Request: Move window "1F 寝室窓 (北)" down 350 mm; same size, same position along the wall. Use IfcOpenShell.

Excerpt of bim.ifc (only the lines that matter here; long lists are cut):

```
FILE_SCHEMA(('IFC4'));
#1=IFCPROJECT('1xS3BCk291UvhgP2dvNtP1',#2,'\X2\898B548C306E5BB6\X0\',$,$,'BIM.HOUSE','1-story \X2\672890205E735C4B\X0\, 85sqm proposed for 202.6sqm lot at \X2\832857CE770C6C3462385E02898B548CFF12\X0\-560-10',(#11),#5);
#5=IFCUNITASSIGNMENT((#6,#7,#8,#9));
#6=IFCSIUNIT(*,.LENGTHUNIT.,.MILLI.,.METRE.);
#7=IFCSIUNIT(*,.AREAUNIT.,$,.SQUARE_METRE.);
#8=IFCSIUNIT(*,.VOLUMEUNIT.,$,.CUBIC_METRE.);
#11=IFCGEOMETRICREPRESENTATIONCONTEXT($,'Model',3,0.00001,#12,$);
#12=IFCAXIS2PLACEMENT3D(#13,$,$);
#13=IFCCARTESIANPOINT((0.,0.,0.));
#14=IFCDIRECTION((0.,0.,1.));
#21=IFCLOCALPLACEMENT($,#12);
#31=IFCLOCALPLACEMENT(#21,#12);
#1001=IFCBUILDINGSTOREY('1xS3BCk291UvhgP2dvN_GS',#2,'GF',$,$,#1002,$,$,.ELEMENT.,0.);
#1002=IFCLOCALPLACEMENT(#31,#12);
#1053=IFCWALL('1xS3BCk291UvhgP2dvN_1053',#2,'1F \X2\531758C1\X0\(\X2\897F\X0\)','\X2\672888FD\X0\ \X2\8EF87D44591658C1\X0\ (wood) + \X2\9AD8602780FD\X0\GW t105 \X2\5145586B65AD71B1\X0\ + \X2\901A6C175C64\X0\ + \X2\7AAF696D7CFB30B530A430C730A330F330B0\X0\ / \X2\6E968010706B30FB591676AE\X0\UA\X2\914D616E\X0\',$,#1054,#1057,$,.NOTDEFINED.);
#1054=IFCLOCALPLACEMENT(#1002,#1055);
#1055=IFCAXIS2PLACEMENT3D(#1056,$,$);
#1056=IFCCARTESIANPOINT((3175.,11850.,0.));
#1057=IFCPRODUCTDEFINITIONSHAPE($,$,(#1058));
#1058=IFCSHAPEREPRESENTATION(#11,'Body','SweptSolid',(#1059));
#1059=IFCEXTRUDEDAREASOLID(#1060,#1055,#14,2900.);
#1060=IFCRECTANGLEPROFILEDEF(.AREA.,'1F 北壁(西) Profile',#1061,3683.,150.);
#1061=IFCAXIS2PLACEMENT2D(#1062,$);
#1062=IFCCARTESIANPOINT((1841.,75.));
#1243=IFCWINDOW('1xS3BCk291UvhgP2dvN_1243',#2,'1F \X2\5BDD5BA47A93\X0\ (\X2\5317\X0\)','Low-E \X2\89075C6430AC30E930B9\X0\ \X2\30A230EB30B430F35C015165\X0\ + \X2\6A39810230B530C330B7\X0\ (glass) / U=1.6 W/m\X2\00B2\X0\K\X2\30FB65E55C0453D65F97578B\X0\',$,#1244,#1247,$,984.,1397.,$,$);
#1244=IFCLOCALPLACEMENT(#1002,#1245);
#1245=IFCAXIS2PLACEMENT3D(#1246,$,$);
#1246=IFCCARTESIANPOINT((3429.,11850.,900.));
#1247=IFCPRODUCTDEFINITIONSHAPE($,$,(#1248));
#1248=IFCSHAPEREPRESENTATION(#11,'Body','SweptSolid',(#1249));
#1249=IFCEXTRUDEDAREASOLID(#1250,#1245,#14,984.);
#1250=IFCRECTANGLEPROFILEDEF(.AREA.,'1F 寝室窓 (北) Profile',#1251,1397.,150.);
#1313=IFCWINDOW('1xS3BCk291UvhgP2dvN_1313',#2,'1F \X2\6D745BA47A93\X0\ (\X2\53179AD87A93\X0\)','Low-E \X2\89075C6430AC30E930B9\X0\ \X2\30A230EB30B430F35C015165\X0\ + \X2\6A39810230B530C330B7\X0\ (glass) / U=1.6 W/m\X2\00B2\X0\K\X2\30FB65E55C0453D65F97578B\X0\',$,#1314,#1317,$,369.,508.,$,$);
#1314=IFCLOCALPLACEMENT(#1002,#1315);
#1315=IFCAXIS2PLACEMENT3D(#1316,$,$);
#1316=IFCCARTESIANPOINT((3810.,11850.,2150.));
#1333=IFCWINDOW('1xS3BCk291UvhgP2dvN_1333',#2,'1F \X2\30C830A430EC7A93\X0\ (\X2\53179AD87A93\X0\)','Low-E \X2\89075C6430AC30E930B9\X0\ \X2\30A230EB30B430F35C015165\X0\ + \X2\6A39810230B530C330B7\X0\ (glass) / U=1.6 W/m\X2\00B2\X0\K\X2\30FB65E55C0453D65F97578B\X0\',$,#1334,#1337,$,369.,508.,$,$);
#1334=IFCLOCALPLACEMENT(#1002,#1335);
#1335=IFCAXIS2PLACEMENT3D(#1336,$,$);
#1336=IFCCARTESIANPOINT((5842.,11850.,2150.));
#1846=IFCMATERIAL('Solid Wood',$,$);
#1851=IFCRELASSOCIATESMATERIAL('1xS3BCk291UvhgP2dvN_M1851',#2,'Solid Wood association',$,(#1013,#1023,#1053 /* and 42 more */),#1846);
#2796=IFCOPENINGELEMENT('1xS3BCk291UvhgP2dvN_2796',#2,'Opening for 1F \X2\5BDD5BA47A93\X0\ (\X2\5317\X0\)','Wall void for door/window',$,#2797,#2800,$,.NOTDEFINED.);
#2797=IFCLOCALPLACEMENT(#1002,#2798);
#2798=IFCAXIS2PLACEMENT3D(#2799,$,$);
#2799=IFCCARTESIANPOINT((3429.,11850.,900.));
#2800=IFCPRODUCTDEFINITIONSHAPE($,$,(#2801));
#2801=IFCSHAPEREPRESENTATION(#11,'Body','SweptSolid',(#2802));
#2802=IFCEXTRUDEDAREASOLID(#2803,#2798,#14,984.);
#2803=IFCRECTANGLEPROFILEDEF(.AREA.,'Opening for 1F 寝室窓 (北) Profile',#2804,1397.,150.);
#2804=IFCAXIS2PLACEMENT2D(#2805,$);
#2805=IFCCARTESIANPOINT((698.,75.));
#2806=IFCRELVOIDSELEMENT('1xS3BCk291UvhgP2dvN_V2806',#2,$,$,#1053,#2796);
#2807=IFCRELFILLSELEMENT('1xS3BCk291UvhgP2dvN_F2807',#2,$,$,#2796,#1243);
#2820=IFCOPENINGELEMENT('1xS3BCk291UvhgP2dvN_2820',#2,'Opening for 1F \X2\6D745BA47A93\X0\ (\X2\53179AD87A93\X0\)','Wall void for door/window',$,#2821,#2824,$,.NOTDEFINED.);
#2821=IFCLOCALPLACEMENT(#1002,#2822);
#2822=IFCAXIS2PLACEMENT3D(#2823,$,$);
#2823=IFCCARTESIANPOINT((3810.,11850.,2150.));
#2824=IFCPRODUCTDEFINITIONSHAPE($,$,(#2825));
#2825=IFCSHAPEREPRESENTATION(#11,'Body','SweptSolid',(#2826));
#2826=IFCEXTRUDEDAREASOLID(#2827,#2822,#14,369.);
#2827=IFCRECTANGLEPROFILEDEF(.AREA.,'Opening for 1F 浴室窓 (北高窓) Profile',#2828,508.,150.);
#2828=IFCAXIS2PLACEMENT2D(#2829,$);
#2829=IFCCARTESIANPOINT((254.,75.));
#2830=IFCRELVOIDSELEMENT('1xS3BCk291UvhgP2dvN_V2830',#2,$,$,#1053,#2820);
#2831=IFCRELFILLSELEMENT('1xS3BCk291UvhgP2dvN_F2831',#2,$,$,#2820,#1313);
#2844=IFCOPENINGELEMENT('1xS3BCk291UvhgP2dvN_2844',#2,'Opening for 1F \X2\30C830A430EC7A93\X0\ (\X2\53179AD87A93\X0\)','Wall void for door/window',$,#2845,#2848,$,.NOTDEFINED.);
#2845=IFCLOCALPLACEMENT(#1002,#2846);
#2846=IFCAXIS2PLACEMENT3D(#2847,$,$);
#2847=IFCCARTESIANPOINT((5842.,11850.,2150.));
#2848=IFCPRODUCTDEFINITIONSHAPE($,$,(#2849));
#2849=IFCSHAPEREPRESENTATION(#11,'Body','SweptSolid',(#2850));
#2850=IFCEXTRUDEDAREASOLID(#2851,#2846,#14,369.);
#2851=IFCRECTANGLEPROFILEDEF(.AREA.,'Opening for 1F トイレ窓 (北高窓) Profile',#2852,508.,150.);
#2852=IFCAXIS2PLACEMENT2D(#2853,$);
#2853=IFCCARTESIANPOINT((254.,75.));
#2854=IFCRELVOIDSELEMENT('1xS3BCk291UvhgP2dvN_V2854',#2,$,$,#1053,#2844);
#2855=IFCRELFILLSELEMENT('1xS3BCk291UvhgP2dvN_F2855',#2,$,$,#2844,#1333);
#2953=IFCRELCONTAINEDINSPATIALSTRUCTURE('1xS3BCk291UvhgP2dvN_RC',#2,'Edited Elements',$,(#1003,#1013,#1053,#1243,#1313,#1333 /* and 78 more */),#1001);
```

```python
import numpy as np
import ifcopenshell
import ifcopenshell.api.geometry
import ifcopenshell.util.placement
import ifcopenshell.util.unit

model = ifcopenshell.open("bim.ifc")
unit_scale = ifcopenshell.util.unit.calculate_unit_scale(model)

window = model.by_id(1243)
opening = window.FillsVoids[0].RelatingOpeningElement
dz = -0.35 / unit_scale

shift = np.array([0.0, 0.0, dz])
# The window is not placed relative to its opening, so move both.
for product in (opening, window):
    matrix = ifcopenshell.util.placement.get_local_placement(product.ObjectPlacement)
    matrix[:3, 3] += shift
    ifcopenshell.api.geometry.edit_object_placement(model, product=product, matrix=matrix, is_si=False)

print(f"moved by {dz * unit_scale:+.3f} m")

model.write("bim-out.ifc")
```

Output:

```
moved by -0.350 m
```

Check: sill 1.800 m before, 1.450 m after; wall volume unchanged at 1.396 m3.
